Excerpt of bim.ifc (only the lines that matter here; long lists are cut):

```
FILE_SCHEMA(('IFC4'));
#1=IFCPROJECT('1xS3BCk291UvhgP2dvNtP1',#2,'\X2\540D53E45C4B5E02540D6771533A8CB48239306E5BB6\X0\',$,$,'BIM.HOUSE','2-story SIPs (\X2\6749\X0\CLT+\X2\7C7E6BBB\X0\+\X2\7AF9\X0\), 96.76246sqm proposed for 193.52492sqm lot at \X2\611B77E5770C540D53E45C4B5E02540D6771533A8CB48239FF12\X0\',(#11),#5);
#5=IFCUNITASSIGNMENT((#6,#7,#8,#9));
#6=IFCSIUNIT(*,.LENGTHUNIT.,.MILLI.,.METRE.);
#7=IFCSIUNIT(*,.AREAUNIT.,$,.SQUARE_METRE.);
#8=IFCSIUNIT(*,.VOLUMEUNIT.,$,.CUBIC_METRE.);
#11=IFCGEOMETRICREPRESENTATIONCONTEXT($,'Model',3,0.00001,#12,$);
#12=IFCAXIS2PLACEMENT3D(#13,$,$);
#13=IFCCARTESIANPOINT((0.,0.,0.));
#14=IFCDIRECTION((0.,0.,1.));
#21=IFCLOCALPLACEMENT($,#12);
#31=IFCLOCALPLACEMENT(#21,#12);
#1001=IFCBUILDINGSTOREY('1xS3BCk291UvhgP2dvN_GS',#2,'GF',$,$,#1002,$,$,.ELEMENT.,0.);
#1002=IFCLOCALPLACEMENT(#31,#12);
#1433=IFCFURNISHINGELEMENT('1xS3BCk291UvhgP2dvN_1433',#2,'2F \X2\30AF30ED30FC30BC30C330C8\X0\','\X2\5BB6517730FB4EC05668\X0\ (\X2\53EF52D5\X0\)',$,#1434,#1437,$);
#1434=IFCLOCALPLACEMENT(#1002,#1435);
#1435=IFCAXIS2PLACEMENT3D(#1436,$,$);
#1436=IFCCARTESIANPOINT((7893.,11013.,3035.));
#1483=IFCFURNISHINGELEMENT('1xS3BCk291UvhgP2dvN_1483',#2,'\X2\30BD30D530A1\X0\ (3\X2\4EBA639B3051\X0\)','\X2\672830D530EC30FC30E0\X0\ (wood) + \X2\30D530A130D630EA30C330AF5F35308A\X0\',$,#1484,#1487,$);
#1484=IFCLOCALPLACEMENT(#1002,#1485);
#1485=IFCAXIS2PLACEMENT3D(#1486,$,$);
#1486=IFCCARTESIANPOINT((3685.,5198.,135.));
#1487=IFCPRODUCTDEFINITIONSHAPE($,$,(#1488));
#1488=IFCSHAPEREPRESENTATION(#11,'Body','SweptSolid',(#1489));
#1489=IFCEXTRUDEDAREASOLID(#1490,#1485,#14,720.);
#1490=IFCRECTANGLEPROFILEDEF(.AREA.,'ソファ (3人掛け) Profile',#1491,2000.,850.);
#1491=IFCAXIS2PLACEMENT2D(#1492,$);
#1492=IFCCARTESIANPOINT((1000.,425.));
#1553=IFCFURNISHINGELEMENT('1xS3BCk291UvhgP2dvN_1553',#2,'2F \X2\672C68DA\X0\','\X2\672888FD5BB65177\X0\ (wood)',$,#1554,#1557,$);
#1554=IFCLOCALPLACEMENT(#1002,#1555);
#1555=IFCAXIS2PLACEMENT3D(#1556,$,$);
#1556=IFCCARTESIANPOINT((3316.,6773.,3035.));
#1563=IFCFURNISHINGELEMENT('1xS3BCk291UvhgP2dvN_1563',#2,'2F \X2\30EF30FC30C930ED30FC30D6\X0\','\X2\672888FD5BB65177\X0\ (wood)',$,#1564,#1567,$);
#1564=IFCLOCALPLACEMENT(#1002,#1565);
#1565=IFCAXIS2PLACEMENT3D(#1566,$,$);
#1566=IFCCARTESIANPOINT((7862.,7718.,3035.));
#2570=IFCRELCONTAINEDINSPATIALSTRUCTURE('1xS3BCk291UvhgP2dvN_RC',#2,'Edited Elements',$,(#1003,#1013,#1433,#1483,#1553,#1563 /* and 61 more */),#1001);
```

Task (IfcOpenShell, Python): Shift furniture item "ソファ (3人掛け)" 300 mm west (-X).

```python
import ifcopenshell
import ifcopenshell.api.geometry
import ifcopenshell.util.placement
import ifcopenshell.util.unit

model = ifcopenshell.open("bim.ifc")
unit_scale = ifcopenshell.util.unit.calculate_unit_scale(model)

item = model.by_guid("1xS3BCk291UvhgP2dvN_1483")
matrix = ifcopenshell.util.placement.get_local_placement(item.ObjectPlacement)
matrix[0, 3] -= 0.3 / unit_scale
ifcopenshell.api.geometry.edit_object_placement(model, product=item, matrix=matrix, is_si=False)

print(ifcopenshell.util.placement.get_local_placement(item.ObjectPlacement).round(3) + 0.0)

model.write("bim_updated.ifc")
```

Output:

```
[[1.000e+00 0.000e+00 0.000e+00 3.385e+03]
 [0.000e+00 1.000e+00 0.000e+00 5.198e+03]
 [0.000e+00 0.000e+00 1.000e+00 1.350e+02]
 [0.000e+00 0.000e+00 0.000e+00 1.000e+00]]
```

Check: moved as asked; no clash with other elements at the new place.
